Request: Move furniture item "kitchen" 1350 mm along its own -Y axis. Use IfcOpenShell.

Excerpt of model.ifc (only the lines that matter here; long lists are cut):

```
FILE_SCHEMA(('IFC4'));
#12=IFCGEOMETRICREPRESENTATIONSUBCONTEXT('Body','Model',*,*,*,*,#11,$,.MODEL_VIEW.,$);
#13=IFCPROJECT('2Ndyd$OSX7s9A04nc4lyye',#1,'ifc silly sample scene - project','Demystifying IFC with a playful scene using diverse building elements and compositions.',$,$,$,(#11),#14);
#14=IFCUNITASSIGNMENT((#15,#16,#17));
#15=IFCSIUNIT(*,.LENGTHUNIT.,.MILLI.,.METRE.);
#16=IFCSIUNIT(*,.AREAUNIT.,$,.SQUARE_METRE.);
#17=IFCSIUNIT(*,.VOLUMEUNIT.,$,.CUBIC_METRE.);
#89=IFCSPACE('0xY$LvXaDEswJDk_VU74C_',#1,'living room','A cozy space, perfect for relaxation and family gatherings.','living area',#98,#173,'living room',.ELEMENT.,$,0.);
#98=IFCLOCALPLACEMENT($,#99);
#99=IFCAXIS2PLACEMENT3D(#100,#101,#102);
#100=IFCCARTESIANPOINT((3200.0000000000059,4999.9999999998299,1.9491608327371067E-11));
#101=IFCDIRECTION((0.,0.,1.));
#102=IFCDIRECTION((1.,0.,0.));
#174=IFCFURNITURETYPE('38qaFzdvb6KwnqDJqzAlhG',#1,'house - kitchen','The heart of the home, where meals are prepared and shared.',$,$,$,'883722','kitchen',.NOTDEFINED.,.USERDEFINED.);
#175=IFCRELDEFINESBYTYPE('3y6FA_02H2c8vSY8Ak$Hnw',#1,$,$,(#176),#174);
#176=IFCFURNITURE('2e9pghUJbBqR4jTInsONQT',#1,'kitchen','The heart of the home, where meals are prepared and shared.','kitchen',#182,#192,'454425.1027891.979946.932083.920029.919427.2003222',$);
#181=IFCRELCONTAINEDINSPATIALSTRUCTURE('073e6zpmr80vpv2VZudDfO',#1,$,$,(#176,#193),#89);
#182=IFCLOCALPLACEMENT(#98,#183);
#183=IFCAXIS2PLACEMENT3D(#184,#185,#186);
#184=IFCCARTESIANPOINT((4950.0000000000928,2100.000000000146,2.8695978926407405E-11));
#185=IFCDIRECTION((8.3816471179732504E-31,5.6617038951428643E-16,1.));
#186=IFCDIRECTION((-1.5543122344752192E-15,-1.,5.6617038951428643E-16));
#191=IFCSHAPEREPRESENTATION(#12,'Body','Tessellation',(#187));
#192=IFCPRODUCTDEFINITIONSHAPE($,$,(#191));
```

```python
import ifcopenshell
import ifcopenshell.api.geometry
import ifcopenshell.util.placement

model = ifcopenshell.open("model.ifc")

item = model.by_id(176)
matrix = ifcopenshell.util.placement.get_local_placement(item.ObjectPlacement)
matrix[:3, 3] -= matrix[:3, 1] * 1350.0
ifcopenshell.api.geometry.edit_object_placement(model, product=item, matrix=matrix, is_si=False)

print(ifcopenshell.util.placement.get_local_placement(item.ObjectPlacement).round(3) + 0.0)

model.write("model_rev.ifc")
```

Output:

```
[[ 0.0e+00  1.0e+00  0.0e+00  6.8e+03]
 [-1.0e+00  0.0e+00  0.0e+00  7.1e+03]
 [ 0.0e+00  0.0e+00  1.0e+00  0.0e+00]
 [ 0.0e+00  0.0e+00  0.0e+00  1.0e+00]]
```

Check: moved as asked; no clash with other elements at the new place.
